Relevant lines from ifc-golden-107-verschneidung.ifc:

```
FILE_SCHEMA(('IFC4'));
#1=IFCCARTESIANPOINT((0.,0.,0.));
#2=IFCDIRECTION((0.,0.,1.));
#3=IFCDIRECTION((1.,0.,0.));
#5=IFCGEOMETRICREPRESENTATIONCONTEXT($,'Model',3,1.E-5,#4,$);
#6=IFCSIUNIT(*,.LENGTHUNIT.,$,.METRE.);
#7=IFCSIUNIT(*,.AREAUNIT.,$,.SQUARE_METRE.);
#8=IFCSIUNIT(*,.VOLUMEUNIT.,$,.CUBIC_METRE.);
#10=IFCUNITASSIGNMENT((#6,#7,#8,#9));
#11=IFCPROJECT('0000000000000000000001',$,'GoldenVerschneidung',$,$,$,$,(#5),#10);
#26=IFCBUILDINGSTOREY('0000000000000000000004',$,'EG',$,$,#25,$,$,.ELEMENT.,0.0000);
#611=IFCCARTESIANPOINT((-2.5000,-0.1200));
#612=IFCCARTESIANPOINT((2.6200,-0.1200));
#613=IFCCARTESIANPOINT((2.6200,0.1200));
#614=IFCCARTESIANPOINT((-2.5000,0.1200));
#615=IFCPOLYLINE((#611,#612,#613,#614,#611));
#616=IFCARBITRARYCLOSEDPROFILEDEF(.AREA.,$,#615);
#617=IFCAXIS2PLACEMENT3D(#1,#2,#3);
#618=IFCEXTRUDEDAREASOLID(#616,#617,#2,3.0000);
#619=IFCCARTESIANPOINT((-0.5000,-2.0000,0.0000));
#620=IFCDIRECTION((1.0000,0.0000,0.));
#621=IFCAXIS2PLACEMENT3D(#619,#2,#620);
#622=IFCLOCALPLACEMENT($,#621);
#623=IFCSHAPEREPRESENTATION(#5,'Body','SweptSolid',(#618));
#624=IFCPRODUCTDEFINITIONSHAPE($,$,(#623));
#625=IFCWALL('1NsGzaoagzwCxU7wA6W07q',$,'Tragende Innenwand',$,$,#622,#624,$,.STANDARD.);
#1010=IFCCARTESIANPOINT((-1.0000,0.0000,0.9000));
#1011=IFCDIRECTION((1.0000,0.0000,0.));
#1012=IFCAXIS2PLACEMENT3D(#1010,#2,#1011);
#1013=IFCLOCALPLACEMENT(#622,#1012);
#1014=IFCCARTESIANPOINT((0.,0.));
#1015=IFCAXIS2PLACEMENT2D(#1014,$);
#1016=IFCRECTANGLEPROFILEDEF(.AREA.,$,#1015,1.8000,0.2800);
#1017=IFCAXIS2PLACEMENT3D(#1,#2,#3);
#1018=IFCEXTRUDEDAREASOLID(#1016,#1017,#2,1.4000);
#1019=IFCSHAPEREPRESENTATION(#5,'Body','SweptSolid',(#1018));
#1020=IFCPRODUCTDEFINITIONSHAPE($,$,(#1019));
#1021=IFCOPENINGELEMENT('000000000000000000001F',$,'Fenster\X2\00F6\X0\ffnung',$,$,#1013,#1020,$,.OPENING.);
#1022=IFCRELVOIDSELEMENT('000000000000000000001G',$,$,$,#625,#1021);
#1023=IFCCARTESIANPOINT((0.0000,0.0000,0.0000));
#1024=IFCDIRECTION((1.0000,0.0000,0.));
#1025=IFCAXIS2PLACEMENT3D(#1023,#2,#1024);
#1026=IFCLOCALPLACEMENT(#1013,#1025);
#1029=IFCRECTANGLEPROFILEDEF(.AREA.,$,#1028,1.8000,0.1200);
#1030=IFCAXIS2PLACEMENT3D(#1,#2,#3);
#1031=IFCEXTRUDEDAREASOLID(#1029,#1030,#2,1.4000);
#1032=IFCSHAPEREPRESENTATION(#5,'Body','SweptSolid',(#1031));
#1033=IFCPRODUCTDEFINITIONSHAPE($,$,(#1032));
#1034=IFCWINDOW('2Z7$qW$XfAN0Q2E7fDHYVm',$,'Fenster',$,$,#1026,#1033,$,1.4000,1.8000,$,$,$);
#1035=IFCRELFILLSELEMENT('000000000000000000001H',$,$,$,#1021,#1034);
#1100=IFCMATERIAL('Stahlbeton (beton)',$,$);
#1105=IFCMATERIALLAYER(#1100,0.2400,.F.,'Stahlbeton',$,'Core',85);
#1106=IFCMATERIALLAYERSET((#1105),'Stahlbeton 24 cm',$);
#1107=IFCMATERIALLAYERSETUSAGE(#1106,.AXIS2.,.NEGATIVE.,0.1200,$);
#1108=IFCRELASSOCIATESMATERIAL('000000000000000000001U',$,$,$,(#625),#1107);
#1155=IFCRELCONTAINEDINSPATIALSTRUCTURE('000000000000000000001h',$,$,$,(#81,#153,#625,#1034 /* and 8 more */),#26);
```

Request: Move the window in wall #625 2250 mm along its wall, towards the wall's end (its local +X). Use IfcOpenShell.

```python
import ifcopenshell
import ifcopenshell.api.geometry
import ifcopenshell.util.placement
import ifcopenshell.util.unit

model = ifcopenshell.open("ifc-golden-107-verschneidung.ifc")
unit_scale = ifcopenshell.util.unit.calculate_unit_scale(model)

window = model.by_guid("2Z7$qW$XfAN0Q2E7fDHYVm")
opening = window.FillsVoids[0].RelatingOpeningElement
wall = opening.VoidsElements[0].RelatingBuildingElement

wall_matrix = ifcopenshell.util.placement.get_local_placement(wall.ObjectPlacement)
shift = wall_matrix[:3, 0] * 2.25 / unit_scale
before = ifcopenshell.util.placement.get_local_placement(window.ObjectPlacement)[:3, 3].copy()

# The window is placed relative to its opening, so it follows when the opening moves.
matrix = ifcopenshell.util.placement.get_local_placement(opening.ObjectPlacement)
matrix[:3, 3] += shift
ifcopenshell.api.geometry.edit_object_placement(
    model, product=opening, matrix=matrix, is_si=False, should_transform_children=True
)

after = ifcopenshell.util.placement.get_local_placement(window.ObjectPlacement)[:3, 3]
print("window moved by", (after - before).round(3) + 0.0)

model.write("ifc-golden-107-verschneidung_updated.ifc")
```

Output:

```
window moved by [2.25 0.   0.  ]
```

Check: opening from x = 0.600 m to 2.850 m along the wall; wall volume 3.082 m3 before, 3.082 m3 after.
